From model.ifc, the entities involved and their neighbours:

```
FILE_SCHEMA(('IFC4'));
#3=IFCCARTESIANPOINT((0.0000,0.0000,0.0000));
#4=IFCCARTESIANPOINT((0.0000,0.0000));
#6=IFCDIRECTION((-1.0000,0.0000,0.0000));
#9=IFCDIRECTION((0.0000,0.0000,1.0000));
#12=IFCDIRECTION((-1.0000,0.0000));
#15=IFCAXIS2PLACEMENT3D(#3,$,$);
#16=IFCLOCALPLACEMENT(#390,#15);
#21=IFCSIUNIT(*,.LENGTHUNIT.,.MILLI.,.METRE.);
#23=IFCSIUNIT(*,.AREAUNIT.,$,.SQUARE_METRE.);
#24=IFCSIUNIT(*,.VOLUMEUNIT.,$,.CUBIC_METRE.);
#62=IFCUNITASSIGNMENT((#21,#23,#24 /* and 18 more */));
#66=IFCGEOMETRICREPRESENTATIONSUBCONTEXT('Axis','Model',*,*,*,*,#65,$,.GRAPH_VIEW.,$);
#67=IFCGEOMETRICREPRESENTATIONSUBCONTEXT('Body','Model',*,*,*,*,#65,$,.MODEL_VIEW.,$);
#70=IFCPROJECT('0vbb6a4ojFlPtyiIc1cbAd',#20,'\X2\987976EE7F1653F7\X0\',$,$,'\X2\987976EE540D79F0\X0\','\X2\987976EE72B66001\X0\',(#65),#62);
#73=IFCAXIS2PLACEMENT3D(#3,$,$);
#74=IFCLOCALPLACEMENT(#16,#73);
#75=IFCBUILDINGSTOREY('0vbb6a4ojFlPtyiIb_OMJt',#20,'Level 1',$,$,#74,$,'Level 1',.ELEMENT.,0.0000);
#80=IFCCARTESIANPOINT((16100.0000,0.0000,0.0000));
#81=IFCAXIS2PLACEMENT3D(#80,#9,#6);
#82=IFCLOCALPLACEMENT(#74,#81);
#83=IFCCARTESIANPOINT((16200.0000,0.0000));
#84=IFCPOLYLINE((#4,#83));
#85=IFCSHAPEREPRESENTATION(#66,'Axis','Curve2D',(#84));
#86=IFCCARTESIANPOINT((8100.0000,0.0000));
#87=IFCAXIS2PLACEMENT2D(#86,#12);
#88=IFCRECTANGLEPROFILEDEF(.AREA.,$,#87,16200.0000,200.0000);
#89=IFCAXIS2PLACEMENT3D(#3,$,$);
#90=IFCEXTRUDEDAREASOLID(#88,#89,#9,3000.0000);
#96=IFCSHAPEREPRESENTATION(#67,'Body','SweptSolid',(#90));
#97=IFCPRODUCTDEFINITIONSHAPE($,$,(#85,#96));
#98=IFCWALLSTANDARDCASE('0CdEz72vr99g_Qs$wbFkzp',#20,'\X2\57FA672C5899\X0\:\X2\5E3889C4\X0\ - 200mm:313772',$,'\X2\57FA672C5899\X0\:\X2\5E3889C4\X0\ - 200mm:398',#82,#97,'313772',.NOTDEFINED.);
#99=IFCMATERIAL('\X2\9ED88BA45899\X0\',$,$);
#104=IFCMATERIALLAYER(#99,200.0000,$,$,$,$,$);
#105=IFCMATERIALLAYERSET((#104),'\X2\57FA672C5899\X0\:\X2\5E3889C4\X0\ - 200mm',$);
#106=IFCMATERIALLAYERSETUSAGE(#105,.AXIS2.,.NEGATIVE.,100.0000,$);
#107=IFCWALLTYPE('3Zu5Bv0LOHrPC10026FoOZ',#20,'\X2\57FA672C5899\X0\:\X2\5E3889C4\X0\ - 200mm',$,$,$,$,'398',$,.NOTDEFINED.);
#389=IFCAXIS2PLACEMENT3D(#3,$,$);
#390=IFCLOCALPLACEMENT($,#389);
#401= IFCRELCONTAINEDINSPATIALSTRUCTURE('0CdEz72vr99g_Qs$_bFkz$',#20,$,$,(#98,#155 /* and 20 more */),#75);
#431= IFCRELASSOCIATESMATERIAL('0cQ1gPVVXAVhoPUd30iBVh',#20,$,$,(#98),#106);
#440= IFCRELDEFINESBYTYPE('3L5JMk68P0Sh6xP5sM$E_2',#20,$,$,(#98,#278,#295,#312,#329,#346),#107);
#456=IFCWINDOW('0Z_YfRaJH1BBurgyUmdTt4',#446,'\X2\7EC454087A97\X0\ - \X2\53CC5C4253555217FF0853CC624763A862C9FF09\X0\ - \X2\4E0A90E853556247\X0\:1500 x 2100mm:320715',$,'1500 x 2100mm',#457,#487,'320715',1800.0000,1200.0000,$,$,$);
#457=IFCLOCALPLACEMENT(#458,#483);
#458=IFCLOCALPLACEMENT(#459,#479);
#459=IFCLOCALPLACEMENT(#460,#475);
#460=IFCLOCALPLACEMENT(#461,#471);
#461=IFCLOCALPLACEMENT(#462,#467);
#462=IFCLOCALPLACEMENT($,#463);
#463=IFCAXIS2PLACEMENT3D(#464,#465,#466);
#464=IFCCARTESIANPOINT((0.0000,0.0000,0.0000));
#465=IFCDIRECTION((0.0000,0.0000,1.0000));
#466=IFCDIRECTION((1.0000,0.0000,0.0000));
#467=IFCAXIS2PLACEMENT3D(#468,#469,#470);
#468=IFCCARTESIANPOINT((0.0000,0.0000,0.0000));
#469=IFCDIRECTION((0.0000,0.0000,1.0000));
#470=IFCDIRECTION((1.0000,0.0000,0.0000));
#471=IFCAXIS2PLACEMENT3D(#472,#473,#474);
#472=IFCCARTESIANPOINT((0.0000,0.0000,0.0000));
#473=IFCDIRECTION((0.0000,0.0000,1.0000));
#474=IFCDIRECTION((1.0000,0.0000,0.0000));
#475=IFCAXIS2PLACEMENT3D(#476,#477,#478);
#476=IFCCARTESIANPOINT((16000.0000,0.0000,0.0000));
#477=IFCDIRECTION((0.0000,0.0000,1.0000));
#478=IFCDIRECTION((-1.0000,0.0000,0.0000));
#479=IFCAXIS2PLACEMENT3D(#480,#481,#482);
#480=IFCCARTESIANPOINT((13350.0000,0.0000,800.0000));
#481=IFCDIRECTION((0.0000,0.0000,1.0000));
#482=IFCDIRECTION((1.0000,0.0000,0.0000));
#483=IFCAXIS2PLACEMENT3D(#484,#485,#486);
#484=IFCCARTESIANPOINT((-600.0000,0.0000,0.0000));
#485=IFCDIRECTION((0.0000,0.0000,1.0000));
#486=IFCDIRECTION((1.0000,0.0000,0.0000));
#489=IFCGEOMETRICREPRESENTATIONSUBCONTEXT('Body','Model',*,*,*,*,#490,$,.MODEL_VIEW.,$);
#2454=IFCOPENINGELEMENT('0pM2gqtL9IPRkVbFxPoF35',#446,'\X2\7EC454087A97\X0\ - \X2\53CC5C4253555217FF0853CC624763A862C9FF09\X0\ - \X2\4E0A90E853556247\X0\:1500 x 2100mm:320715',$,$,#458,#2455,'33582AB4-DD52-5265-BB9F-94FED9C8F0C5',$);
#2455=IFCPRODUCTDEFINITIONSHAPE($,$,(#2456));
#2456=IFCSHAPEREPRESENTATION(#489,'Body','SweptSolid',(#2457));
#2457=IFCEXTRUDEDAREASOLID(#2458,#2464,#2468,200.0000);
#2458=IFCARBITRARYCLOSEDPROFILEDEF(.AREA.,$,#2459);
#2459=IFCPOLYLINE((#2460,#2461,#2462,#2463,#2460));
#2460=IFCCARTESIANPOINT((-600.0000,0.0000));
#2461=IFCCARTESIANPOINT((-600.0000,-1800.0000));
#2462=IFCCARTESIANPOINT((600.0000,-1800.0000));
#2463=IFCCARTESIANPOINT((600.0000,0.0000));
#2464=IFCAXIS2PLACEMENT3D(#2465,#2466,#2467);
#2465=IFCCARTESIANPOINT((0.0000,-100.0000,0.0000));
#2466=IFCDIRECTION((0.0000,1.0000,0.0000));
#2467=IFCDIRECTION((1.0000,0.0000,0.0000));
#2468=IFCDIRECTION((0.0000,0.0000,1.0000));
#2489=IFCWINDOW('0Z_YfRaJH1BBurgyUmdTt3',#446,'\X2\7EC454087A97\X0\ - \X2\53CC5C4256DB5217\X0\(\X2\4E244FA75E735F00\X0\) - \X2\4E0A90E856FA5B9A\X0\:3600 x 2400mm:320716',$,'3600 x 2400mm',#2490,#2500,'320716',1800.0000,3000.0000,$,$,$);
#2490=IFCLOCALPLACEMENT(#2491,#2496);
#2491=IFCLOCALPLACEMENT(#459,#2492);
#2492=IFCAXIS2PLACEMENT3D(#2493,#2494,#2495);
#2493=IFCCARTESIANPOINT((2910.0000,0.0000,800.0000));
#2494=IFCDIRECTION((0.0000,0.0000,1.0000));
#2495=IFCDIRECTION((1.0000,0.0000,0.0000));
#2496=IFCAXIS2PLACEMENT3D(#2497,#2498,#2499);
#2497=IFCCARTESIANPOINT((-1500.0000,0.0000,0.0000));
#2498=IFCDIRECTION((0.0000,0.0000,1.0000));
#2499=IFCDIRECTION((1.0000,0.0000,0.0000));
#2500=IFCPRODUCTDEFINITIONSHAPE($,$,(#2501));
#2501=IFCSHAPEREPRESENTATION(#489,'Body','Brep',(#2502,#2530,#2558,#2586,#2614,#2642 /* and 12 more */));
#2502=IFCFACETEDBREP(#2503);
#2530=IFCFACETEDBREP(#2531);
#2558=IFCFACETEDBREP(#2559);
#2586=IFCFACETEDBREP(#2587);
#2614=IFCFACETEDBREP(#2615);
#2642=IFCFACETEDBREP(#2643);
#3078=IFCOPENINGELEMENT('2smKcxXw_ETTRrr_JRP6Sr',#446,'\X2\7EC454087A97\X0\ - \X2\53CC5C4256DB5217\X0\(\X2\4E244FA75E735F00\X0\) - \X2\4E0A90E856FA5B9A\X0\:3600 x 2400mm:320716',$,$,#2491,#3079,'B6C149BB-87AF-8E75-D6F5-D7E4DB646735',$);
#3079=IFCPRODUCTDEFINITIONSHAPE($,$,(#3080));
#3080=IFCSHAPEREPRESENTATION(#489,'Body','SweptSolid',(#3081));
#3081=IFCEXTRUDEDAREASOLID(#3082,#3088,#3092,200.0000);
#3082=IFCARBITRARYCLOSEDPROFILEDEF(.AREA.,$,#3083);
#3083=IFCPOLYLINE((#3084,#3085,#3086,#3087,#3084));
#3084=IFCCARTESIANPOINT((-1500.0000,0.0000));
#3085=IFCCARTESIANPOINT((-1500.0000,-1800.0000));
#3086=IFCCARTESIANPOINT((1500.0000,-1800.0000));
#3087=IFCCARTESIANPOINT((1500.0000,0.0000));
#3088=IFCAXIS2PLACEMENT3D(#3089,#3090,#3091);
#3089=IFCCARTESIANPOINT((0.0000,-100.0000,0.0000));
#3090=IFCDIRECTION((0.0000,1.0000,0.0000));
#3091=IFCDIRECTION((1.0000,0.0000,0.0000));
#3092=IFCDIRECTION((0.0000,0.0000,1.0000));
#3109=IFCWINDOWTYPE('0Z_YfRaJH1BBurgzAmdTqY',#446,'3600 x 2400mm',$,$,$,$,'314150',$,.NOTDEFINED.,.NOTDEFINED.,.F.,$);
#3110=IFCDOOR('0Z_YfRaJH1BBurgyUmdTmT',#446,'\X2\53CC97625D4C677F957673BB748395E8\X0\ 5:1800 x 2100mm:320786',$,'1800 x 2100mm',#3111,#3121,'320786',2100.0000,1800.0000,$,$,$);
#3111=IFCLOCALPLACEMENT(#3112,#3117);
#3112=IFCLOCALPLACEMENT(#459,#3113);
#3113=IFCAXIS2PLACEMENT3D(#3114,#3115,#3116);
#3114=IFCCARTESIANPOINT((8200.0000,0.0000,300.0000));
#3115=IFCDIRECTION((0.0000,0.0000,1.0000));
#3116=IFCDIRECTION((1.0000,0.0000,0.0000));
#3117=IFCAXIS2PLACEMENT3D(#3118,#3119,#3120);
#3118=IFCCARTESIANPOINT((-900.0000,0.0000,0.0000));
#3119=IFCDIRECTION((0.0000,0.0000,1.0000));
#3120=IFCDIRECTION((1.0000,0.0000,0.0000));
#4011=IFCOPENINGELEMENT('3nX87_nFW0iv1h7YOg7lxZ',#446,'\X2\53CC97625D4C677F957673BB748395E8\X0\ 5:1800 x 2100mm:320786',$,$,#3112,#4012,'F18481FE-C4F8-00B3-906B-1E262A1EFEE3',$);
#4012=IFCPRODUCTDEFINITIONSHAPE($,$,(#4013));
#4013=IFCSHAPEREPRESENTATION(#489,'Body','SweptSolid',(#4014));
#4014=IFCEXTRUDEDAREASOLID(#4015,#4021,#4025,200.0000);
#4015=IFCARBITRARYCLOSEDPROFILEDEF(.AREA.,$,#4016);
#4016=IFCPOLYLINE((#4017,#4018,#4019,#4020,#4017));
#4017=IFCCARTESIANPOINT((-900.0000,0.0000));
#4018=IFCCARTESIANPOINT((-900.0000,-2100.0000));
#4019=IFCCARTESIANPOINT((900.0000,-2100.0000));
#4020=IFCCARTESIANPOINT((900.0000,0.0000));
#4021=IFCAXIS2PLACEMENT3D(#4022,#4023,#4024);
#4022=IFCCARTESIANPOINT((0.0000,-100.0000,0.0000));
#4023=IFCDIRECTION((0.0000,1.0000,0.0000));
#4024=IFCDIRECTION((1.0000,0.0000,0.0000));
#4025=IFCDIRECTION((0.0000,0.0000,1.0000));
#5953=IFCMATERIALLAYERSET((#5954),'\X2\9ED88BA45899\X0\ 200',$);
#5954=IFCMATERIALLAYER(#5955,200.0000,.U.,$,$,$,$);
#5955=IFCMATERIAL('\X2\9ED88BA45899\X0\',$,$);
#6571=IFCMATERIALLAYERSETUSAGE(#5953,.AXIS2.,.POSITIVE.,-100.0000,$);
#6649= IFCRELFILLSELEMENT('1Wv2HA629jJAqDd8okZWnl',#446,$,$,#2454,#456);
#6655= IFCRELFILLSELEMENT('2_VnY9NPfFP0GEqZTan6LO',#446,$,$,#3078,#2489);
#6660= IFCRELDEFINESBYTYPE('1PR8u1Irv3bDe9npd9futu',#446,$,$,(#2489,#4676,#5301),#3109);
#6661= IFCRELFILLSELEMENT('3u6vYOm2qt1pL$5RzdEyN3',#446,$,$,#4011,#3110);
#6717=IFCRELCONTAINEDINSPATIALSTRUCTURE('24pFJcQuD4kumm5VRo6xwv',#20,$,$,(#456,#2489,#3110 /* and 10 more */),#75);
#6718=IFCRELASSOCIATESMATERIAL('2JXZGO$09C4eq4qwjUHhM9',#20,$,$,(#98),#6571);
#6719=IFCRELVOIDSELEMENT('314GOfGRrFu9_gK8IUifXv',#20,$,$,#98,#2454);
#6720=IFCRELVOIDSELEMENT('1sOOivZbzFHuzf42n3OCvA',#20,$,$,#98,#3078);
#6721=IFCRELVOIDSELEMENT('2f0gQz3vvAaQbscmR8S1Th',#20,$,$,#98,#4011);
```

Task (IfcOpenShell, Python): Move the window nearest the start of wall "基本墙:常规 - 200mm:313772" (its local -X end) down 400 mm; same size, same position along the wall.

```python
import numpy as np
import ifcopenshell
import ifcopenshell.api.geometry
import ifcopenshell.util.placement
import ifcopenshell.util.unit

model = ifcopenshell.open("model.ifc")
unit_scale = ifcopenshell.util.unit.calculate_unit_scale(model)

window = model.by_guid("0Z_YfRaJH1BBurgyUmdTt3")
opening = window.FillsVoids[0].RelatingOpeningElement
dz = -0.4 / unit_scale

shift = np.array([0.0, 0.0, dz])
# The window is placed relative to its opening, so it follows when the opening moves.
matrix = ifcopenshell.util.placement.get_local_placement(opening.ObjectPlacement)
matrix[:3, 3] += shift
ifcopenshell.api.geometry.edit_object_placement(
    model, product=opening, matrix=matrix, is_si=False, should_transform_children=True
)

print(f"moved by {dz * unit_scale:+.3f} m")

model.write("model_edited.ifc")
```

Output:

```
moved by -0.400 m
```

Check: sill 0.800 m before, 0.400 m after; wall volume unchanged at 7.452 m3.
